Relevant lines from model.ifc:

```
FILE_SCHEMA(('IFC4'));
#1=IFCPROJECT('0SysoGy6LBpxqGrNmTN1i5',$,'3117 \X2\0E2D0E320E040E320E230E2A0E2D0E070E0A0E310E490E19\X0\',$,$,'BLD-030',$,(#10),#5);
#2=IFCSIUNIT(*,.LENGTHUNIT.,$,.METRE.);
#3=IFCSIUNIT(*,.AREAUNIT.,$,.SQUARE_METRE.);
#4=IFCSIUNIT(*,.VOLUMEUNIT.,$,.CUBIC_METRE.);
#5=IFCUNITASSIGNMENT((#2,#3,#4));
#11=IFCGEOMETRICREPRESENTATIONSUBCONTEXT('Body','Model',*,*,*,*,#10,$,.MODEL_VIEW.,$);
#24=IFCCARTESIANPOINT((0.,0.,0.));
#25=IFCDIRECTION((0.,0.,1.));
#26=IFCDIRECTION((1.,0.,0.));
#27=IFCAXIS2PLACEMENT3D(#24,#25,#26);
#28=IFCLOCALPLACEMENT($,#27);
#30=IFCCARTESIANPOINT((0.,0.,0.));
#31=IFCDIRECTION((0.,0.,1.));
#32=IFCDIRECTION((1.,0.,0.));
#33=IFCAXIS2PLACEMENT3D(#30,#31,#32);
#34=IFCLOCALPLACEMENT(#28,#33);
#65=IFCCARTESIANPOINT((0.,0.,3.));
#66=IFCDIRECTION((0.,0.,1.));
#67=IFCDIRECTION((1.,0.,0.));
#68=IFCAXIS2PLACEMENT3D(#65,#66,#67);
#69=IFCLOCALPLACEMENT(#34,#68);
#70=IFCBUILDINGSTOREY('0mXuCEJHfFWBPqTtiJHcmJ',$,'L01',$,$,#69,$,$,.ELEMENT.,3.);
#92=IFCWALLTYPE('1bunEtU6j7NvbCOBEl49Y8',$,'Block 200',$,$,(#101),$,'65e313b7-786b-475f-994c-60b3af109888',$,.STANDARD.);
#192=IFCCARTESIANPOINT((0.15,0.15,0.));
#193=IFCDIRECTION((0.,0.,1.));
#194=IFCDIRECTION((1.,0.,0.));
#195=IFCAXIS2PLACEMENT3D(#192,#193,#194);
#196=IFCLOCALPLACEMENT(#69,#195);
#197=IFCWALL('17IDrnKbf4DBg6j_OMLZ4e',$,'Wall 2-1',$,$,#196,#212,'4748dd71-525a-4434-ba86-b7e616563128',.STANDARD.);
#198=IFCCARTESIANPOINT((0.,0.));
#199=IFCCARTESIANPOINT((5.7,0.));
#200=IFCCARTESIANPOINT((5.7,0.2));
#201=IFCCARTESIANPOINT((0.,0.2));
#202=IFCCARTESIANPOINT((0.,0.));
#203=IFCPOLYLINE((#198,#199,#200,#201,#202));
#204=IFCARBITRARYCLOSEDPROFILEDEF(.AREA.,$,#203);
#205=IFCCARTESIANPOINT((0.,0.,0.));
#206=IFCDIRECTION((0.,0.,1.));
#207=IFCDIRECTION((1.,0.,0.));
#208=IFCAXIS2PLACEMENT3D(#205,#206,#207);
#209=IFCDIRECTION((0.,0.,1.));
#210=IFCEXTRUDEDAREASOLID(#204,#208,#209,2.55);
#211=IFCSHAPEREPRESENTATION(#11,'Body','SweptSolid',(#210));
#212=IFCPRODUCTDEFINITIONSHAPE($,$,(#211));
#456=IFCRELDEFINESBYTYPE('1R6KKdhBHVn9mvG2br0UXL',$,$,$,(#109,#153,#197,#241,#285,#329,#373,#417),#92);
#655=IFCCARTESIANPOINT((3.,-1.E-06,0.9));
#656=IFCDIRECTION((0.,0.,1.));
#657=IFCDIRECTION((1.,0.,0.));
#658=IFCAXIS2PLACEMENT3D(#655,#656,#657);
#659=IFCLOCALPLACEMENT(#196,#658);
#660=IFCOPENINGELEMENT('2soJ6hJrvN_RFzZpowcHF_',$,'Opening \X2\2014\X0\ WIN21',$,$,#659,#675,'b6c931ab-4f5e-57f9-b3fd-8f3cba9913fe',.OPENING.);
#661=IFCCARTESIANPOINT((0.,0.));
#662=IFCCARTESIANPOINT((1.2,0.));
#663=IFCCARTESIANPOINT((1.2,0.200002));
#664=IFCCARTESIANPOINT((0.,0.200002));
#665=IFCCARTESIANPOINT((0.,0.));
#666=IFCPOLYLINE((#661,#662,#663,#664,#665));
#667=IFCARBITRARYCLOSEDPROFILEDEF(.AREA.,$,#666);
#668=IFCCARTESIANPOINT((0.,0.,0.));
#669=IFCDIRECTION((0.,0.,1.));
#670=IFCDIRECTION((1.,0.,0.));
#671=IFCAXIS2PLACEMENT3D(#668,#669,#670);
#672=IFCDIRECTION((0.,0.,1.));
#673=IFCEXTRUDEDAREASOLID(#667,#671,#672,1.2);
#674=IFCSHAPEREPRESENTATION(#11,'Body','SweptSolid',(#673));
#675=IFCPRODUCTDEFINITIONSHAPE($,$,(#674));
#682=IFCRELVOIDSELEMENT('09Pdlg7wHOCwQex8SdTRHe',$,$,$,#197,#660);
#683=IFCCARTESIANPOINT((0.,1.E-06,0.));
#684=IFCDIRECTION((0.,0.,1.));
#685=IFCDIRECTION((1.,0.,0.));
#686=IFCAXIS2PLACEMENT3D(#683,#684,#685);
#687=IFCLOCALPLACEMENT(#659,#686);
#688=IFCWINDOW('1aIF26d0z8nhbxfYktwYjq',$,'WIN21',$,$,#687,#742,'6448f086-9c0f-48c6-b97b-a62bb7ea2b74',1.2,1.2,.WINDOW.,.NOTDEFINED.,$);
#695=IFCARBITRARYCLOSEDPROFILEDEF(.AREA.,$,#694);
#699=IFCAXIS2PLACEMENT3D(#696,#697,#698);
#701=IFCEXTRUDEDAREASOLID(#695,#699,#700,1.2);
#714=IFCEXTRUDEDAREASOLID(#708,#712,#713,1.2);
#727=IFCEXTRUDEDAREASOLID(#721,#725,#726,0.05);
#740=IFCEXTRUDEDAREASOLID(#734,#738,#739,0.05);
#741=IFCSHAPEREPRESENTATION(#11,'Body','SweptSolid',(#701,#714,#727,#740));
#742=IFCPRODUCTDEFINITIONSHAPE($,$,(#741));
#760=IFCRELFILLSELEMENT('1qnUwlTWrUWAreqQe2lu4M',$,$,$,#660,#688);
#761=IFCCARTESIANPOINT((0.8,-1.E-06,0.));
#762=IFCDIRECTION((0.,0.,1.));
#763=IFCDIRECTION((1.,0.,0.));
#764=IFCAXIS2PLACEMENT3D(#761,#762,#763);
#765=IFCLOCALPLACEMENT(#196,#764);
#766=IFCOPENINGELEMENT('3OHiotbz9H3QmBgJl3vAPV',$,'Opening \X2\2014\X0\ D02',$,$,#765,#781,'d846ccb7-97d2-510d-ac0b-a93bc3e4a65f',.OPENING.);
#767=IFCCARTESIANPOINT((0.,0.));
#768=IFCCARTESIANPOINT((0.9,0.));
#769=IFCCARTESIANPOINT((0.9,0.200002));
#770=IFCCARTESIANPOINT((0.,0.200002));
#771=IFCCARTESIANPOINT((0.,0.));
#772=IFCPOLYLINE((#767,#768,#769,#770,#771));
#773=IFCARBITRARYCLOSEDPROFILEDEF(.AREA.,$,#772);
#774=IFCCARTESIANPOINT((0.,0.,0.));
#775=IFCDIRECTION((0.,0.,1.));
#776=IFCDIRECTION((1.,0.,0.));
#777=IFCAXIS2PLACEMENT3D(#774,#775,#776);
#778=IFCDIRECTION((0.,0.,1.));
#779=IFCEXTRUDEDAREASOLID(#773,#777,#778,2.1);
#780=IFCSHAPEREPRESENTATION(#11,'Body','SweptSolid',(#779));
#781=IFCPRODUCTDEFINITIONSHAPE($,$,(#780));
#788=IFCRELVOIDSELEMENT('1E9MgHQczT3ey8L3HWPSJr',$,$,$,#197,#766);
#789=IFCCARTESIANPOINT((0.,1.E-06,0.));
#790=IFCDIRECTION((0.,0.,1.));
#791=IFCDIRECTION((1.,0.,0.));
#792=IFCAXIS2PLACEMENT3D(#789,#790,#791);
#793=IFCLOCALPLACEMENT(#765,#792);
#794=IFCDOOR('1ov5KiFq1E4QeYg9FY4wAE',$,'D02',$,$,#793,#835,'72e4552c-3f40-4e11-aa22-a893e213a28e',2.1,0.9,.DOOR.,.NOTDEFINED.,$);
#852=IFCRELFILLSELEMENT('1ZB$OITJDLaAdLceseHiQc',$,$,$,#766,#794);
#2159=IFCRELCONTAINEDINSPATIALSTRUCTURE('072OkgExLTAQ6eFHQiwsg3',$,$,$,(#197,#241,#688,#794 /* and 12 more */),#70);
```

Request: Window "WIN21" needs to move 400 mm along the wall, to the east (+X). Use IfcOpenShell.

```python
import ifcopenshell
import ifcopenshell.api.geometry
import ifcopenshell.util.placement
import ifcopenshell.util.unit

model = ifcopenshell.open("model.ifc")
unit_scale = ifcopenshell.util.unit.calculate_unit_scale(model)

window = model.by_guid("1aIF26d0z8nhbxfYktwYjq")
opening = window.FillsVoids[0].RelatingOpeningElement
wall = opening.VoidsElements[0].RelatingBuildingElement

wall_matrix = ifcopenshell.util.placement.get_local_placement(wall.ObjectPlacement)
shift = wall_matrix[:3, 0] * 0.4 / unit_scale
before = ifcopenshell.util.placement.get_local_placement(window.ObjectPlacement)[:3, 3].copy()

# The window is placed relative to its opening, so it follows when the opening moves.
matrix = ifcopenshell.util.placement.get_local_placement(opening.ObjectPlacement)
matrix[:3, 3] += shift
ifcopenshell.api.geometry.edit_object_placement(
    model, product=opening, matrix=matrix, is_si=False, should_transform_children=True
)

after = ifcopenshell.util.placement.get_local_placement(window.ObjectPlacement)[:3, 3]
print("window moved by", (after - before).round(3) + 0.0)

model.write("model_rev.ifc")
```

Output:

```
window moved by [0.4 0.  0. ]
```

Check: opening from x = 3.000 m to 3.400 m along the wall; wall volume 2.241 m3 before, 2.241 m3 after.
